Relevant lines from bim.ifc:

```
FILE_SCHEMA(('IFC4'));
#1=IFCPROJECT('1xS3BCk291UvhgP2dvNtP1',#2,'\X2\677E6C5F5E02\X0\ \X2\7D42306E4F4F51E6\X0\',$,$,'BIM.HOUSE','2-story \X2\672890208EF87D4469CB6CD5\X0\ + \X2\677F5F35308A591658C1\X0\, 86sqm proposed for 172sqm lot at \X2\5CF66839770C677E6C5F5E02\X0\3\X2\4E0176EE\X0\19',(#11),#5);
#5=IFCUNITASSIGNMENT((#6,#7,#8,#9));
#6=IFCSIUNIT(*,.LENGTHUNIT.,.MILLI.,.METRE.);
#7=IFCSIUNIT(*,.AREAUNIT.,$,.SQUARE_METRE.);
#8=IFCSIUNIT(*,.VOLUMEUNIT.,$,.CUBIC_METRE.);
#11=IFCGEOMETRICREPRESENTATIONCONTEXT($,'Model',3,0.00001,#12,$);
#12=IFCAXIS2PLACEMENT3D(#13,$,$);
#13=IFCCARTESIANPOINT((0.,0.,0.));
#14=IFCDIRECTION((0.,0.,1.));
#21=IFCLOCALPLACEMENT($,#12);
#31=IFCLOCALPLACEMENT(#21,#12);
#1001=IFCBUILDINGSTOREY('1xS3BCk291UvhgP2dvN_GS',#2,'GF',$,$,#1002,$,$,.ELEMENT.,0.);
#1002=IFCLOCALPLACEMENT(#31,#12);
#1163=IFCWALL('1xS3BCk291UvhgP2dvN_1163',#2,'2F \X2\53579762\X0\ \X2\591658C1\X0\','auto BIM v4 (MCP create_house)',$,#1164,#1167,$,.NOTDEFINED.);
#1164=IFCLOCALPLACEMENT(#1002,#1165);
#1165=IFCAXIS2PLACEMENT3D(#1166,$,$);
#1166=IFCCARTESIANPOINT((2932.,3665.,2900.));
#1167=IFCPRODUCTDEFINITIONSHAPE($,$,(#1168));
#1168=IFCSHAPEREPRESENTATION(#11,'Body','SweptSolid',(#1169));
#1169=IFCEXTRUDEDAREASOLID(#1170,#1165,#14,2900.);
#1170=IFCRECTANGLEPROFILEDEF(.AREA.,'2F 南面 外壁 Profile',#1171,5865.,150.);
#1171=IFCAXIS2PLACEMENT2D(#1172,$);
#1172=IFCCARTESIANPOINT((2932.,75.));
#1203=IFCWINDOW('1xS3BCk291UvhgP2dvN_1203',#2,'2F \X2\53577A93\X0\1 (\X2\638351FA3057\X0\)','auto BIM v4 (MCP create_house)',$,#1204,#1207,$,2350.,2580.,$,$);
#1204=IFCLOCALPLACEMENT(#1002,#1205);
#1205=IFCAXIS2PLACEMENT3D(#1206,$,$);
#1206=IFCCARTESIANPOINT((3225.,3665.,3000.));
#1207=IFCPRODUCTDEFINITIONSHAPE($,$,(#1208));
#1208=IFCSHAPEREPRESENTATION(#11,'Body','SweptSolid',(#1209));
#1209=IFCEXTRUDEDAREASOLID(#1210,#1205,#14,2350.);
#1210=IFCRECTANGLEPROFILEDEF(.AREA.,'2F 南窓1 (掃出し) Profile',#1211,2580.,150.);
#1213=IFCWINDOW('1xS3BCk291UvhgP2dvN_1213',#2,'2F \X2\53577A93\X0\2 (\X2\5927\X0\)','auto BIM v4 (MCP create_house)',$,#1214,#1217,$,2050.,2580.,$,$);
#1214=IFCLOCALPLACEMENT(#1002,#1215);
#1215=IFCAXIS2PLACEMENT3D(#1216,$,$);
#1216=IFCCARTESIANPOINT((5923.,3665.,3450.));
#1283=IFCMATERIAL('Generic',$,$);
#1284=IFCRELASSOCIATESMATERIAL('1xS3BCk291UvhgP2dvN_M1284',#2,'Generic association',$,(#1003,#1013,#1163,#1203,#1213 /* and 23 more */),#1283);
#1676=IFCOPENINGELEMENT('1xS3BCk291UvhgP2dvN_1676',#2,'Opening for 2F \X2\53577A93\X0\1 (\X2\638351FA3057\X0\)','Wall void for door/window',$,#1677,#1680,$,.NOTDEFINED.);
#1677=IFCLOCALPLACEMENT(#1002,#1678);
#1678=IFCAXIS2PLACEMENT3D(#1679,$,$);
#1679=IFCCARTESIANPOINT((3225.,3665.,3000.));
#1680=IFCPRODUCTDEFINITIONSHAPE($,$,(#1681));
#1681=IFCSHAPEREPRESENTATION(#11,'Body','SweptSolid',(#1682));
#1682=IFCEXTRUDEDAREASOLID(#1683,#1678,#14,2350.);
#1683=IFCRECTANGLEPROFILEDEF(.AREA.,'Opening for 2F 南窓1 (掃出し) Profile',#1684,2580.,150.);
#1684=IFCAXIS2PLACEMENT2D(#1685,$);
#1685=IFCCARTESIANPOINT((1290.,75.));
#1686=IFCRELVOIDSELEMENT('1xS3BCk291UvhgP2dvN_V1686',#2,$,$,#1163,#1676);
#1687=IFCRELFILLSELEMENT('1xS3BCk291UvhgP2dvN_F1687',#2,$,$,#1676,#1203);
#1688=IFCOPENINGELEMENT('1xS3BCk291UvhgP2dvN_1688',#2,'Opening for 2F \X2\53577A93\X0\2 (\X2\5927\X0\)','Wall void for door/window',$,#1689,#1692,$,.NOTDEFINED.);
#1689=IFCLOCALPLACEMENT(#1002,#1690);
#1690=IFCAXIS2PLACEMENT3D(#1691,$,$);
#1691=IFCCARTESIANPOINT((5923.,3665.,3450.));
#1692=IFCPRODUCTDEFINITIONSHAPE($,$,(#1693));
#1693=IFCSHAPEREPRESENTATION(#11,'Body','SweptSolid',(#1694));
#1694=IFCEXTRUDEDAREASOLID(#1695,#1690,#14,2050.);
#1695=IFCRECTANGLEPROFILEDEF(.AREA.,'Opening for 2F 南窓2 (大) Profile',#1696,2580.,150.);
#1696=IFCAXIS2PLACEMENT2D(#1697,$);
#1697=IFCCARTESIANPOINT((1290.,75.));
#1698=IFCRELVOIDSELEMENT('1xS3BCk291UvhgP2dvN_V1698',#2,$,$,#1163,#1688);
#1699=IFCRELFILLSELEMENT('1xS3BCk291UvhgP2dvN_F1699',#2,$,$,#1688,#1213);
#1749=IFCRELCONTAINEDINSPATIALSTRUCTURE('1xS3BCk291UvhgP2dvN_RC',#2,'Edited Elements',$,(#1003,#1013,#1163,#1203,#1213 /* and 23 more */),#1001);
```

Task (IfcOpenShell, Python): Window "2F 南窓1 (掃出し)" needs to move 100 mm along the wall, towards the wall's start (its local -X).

```python
import ifcopenshell
import ifcopenshell.api.geometry
import ifcopenshell.util.placement
import ifcopenshell.util.unit

model = ifcopenshell.open("bim.ifc")
unit_scale = ifcopenshell.util.unit.calculate_unit_scale(model)

window = model.by_guid("1xS3BCk291UvhgP2dvN_1203")
opening = window.FillsVoids[0].RelatingOpeningElement
wall = opening.VoidsElements[0].RelatingBuildingElement

wall_matrix = ifcopenshell.util.placement.get_local_placement(wall.ObjectPlacement)
shift = wall_matrix[:3, 0] * -0.1 / unit_scale
before = ifcopenshell.util.placement.get_local_placement(window.ObjectPlacement)[:3, 3].copy()

# The window is not placed relative to its opening, so move both.
for product in (opening, window):
    matrix = ifcopenshell.util.placement.get_local_placement(product.ObjectPlacement)
    matrix[:3, 3] += shift
    ifcopenshell.api.geometry.edit_object_placement(model, product=product, matrix=matrix, is_si=False)

after = ifcopenshell.util.placement.get_local_placement(window.ObjectPlacement)[:3, 3]
print("window moved by", (after - before).round(3) + 0.0)

model.write("bim_v2.ifc")
```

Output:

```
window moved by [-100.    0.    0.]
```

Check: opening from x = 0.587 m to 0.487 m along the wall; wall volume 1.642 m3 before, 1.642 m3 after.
